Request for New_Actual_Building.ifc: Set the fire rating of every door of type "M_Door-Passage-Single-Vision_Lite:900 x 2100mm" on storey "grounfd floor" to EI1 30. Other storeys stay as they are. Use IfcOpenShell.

First a look at what the model holds.

```python
import ifcopenshell
import ifcopenshell.util.element

model = ifcopenshell.open("New_Actual_Building.ifc")
print(model.schema)
storey = next(s for s in model.by_type("IfcBuildingStorey") if s.Name == "grounfd floor")
doors = [e for e in ifcopenshell.util.element.get_decomposition(storey) if e.is_a("IfcDoor")]
seen = {}
for e in doors:
    element_type = ifcopenshell.util.element.get_type(e)
    key = (element_type.Name if element_type != e and element_type else None, ifcopenshell.util.element.get_pset(e, "Pset_DoorCommon", "FireRating"))
    seen[key] = seen.get(key, 0) + 1
for (name, value), count in sorted(seen.items(), key=str):
    print(count, "x", name, "|", value)
```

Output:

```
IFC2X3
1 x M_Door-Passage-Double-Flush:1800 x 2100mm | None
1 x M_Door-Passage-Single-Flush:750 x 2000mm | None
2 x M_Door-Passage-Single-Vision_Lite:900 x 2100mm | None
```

```python
import ifcopenshell
import ifcopenshell.api.pset
import ifcopenshell.util.element

model = ifcopenshell.open("New_Actual_Building.ifc")

storey = next(s for s in model.by_type("IfcBuildingStorey") if s.Name == "grounfd floor")
doors = [e for e in ifcopenshell.util.element.get_decomposition(storey) if e.is_a("IfcDoor")]

count = 0
for e in doors:
    element_type = ifcopenshell.util.element.get_type(e)
    if element_type in (None, e) or element_type.Name != "M_Door-Passage-Single-Vision_Lite:900 x 2100mm":
        continue
    # add_pset returns the element's existing set when there is one.
    pset = ifcopenshell.api.pset.add_pset(model, product=e, name="Pset_DoorCommon")
    ifcopenshell.api.pset.edit_pset(model, pset=pset, properties={"FireRating": "EI1 30"})
    count += 1

print(count, "doors updated")

model.write("New_Actual_Building_edited.ifc")
```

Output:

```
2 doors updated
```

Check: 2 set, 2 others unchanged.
